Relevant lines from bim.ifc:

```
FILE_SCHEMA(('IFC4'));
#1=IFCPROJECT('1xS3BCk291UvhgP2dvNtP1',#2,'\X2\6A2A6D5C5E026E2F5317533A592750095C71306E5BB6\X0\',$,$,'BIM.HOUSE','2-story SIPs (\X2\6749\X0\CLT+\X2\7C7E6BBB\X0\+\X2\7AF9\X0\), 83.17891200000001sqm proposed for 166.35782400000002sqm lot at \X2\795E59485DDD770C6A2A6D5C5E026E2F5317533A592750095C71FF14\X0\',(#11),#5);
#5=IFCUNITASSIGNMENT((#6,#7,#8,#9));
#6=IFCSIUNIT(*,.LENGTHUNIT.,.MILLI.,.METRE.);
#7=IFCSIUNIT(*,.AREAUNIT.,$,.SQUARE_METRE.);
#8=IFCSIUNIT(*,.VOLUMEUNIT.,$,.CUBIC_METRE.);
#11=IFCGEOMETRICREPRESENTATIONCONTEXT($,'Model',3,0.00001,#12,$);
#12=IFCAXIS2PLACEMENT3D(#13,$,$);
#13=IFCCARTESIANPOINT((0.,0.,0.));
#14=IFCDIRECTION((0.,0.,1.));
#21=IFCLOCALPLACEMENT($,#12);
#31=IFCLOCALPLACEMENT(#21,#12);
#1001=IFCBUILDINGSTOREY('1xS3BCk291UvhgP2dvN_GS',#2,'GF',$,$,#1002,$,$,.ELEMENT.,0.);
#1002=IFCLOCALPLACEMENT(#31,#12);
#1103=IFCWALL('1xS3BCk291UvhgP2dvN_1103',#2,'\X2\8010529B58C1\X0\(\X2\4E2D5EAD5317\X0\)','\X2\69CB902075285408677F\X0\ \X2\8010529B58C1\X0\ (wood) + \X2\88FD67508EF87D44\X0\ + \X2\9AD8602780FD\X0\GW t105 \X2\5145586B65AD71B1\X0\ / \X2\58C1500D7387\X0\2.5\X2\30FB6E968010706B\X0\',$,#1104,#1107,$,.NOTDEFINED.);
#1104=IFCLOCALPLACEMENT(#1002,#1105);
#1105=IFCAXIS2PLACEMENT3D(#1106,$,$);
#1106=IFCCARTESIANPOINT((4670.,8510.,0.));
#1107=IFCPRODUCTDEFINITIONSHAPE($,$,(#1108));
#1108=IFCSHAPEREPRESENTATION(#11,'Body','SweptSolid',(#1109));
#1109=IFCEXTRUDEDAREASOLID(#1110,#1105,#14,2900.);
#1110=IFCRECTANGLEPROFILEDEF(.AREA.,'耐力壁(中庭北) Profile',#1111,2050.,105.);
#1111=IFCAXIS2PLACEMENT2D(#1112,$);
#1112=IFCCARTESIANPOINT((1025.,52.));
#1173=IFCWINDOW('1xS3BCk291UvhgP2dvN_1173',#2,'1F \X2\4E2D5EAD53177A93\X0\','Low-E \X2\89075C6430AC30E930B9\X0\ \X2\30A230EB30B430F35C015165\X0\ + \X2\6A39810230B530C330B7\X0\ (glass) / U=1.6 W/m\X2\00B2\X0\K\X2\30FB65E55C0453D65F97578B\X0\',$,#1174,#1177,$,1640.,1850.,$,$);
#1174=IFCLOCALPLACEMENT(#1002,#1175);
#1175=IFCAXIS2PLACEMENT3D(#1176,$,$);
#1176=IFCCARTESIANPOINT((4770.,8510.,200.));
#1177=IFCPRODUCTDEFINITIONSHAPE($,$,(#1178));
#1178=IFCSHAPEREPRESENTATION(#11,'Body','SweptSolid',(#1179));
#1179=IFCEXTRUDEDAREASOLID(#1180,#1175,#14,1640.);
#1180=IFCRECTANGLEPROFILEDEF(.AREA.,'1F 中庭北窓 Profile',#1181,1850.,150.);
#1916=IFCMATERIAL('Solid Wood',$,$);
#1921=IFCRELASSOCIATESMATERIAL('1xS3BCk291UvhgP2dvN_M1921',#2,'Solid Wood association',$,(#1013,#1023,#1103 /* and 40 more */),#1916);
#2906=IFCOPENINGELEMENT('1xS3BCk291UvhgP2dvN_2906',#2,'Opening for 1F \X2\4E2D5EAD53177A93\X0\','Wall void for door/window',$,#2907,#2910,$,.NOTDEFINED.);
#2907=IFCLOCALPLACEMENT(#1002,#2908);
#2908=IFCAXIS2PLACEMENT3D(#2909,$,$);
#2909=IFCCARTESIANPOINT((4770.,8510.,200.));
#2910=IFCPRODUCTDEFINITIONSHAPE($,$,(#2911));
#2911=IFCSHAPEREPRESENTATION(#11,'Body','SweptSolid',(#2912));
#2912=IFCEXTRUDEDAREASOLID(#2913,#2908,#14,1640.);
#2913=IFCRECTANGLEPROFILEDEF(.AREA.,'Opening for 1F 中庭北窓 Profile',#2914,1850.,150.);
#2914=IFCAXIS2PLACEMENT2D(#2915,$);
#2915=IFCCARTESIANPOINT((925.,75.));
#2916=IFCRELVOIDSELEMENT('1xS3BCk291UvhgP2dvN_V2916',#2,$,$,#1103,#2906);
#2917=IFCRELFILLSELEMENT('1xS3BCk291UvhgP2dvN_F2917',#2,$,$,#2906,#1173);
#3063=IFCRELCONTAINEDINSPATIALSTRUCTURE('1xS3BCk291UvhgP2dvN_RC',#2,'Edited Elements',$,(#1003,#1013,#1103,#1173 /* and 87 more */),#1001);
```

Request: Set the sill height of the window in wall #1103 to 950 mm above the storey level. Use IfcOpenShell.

```python
import numpy as np
import ifcopenshell
import ifcopenshell.api.geometry
import ifcopenshell.geom
import ifcopenshell.util.element
import ifcopenshell.util.placement
import ifcopenshell.util.shape
import ifcopenshell.util.unit

model = ifcopenshell.open("bim.ifc")
unit_scale = ifcopenshell.util.unit.calculate_unit_scale(model)

window = model.by_guid("1xS3BCk291UvhgP2dvN_1173")
opening = window.FillsVoids[0].RelatingOpeningElement
storey = ifcopenshell.util.element.get_container(window, ifc_class="IfcBuildingStorey")
level = ifcopenshell.util.placement.get_local_placement(storey.ObjectPlacement)[2, 3]

# The opening's origin need not be at the sill, so measure its lowest point.
shape = ifcopenshell.geom.create_shape(ifcopenshell.geom.settings(), opening)
bottom = ifcopenshell.util.shape.get_shape_bottom_elevation(shape, shape.geometry) / unit_scale
dz = level + 0.95 / unit_scale - bottom

shift = np.array([0.0, 0.0, dz])
# The window is not placed relative to its opening, so move both.
for product in (opening, window):
    matrix = ifcopenshell.util.placement.get_local_placement(product.ObjectPlacement)
    matrix[:3, 3] += shift
    ifcopenshell.api.geometry.edit_object_placement(model, product=product, matrix=matrix, is_si=False)

print(f"moved by {dz * unit_scale:+.3f} m")

model.write("bim_v2.ifc")
```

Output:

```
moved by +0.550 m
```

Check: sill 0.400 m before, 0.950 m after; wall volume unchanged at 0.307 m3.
